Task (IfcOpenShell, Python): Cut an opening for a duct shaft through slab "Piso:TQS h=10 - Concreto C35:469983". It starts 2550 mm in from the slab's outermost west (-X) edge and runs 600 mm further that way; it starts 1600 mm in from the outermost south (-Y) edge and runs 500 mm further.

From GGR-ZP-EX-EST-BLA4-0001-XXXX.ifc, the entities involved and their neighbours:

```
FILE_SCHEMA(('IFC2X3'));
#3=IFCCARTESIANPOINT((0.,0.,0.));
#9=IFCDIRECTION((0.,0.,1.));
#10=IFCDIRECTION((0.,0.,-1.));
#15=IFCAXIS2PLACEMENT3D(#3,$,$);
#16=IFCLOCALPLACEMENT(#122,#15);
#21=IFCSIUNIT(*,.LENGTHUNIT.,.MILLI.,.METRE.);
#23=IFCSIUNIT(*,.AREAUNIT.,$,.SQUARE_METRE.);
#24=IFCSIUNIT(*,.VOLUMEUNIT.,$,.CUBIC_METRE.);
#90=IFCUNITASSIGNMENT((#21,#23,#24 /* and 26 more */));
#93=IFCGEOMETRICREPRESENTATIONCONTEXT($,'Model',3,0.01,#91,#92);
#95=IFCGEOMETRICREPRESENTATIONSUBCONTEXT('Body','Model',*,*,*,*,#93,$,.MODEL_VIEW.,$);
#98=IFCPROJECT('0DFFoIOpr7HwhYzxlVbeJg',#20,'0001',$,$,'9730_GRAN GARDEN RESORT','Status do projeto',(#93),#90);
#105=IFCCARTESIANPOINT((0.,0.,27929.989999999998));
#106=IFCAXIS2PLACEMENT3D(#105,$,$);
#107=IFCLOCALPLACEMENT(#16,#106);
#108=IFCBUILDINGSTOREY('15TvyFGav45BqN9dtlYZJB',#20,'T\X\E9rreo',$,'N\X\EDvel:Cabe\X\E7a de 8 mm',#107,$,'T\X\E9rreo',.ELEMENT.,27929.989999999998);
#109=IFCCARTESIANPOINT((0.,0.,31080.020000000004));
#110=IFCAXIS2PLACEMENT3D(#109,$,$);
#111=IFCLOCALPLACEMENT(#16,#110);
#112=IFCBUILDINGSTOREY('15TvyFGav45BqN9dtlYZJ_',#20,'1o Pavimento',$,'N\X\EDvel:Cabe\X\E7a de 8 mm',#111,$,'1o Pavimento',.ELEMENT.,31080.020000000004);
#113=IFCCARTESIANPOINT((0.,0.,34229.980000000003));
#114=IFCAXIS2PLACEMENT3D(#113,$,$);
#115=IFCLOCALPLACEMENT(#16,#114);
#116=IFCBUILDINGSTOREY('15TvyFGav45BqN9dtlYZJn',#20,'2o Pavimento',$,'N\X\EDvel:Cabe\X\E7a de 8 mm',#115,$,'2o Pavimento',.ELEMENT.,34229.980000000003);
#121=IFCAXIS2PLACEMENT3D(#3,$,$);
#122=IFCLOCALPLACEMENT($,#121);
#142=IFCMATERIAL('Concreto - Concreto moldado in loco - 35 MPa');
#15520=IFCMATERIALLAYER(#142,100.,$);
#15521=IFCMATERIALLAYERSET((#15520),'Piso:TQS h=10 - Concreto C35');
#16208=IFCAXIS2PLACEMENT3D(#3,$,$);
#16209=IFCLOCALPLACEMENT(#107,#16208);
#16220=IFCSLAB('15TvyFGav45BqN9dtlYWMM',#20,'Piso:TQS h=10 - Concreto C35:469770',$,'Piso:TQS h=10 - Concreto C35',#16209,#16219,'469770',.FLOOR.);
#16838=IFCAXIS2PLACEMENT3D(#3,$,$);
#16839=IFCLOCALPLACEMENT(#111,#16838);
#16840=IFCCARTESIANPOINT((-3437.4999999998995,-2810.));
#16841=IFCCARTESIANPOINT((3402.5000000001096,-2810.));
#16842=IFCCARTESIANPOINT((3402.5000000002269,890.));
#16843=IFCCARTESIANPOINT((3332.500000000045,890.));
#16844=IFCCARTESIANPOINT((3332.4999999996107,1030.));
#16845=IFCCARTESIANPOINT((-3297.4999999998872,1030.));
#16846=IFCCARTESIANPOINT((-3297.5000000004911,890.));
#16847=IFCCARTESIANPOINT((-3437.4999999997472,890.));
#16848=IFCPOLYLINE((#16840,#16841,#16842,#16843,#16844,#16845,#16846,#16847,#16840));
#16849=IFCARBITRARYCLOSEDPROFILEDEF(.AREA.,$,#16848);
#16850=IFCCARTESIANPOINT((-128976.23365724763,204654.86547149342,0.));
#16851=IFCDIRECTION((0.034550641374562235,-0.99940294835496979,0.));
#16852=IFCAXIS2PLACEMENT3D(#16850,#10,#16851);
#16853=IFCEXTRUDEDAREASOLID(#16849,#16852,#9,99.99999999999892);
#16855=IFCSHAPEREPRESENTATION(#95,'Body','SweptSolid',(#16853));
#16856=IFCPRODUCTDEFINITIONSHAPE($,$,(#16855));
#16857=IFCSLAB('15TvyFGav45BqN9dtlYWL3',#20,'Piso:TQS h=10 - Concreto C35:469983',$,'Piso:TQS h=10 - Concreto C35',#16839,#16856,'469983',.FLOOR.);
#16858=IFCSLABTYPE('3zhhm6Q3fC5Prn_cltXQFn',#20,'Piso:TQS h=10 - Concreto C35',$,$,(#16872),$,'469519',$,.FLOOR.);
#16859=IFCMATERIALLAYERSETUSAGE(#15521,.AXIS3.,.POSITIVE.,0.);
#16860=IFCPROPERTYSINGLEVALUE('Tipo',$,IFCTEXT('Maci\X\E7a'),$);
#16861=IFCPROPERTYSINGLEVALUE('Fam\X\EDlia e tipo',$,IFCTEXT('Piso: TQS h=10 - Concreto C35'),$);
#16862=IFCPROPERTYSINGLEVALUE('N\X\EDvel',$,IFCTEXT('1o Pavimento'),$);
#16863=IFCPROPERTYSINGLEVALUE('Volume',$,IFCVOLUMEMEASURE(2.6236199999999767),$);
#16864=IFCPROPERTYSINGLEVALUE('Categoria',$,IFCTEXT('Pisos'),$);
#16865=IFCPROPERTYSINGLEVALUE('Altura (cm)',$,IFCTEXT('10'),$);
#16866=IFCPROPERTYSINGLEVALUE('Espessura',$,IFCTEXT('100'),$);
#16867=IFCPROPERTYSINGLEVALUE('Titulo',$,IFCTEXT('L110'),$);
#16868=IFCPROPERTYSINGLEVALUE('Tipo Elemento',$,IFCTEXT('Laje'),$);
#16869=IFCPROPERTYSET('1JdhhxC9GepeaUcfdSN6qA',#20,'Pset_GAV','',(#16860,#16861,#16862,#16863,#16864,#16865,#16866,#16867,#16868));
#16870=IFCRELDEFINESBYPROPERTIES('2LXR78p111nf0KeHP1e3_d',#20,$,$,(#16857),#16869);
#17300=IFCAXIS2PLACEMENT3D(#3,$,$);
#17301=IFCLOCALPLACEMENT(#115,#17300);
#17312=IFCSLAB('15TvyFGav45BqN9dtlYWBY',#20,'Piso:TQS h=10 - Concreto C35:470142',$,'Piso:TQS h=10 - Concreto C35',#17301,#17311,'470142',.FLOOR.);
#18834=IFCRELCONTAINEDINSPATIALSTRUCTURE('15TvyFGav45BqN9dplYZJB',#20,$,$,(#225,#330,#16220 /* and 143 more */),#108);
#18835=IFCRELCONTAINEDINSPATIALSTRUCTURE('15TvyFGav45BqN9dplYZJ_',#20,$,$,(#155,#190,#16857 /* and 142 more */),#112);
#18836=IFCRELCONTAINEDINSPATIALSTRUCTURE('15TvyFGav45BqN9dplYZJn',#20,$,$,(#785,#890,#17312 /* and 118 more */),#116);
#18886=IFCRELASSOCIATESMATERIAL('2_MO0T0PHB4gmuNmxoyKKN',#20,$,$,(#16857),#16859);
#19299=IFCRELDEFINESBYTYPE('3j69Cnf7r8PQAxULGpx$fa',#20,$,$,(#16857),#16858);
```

```python
import numpy as np
import ifcopenshell
import ifcopenshell.api.feature
import ifcopenshell.api.geometry
import ifcopenshell.api.pset
import ifcopenshell.api.root
import ifcopenshell.geom
import ifcopenshell.util.element
import ifcopenshell.util.placement
import ifcopenshell.util.representation
import ifcopenshell.util.shape
import ifcopenshell.util.unit

model = ifcopenshell.open("GGR-ZP-EX-EST-BLA4-0001-XXXX.ifc")
unit_scale = ifcopenshell.util.unit.calculate_unit_scale(model)
volume_scale = ifcopenshell.util.unit.calculate_unit_scale(model, "VOLUMEUNIT")
settings = ifcopenshell.geom.settings()


def volume(element):
    """Net volume in cubic metres, openings subtracted."""
    shape = ifcopenshell.geom.create_shape(settings, element)
    return ifcopenshell.util.shape.get_volume(shape.geometry)


slab = model.by_guid("15TvyFGav45BqN9dtlYWL3")
before = volume(slab)

# Extent in the slab's own axes, in metres. The edges named are its -X and -Y sides.
slab_shape = ifcopenshell.geom.create_shape(settings, slab)
vertices = ifcopenshell.util.shape.get_vertices(slab_shape.geometry)
x_min, y_min, bottom = vertices.min(axis=0)
top = vertices[:, 2].max()

opening = ifcopenshell.api.root.create_entity(model, ifc_class="IfcOpeningElement", name="Duct shaft opening")
context = ifcopenshell.util.representation.get_context(model, "Model", "Body", "MODEL_VIEW")
width, depth = 0.6, 0.5
outline = [(0.0, 0.0), (width, 0.0), (width, depth), (0.0, depth), (0.0, 0.0)]
# Overshoot both faces by 50 mm so the cut is clean.
shape = ifcopenshell.api.geometry.add_slab_representation(
    model, context=context, depth=top - bottom + 0.1, polyline=outline
)
ifcopenshell.api.geometry.assign_representation(model, product=opening, representation=shape)

matrix = ifcopenshell.util.placement.get_local_placement(slab.ObjectPlacement)
matrix[:, 3] = matrix @ np.append(np.array([x_min + 2.55, y_min + 1.6, bottom - 0.05]) / unit_scale, 1.0)
ifcopenshell.api.geometry.edit_object_placement(model, product=opening, matrix=matrix, is_si=False)
ifcopenshell.api.feature.add_feature(model, feature=opening, element=slab)

after = volume(slab)

# Update the slab's stored quantities.
pset = model.by_id(ifcopenshell.util.element.get_pset(slab, "Pset_GAV", should_inherit=False)["id"])
ifcopenshell.api.pset.edit_pset(model, pset=pset, properties={
    "Volume": model.create_entity("IfcVolumeMeasure", after / volume_scale),
})

print(f"slab volume {before:.3f} -> {after:.3f} m3")

model.write("GGR-ZP-EX-EST-BLA4-0001-XXXX_v2.ifc")
```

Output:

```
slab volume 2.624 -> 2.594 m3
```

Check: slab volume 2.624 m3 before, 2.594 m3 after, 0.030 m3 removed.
